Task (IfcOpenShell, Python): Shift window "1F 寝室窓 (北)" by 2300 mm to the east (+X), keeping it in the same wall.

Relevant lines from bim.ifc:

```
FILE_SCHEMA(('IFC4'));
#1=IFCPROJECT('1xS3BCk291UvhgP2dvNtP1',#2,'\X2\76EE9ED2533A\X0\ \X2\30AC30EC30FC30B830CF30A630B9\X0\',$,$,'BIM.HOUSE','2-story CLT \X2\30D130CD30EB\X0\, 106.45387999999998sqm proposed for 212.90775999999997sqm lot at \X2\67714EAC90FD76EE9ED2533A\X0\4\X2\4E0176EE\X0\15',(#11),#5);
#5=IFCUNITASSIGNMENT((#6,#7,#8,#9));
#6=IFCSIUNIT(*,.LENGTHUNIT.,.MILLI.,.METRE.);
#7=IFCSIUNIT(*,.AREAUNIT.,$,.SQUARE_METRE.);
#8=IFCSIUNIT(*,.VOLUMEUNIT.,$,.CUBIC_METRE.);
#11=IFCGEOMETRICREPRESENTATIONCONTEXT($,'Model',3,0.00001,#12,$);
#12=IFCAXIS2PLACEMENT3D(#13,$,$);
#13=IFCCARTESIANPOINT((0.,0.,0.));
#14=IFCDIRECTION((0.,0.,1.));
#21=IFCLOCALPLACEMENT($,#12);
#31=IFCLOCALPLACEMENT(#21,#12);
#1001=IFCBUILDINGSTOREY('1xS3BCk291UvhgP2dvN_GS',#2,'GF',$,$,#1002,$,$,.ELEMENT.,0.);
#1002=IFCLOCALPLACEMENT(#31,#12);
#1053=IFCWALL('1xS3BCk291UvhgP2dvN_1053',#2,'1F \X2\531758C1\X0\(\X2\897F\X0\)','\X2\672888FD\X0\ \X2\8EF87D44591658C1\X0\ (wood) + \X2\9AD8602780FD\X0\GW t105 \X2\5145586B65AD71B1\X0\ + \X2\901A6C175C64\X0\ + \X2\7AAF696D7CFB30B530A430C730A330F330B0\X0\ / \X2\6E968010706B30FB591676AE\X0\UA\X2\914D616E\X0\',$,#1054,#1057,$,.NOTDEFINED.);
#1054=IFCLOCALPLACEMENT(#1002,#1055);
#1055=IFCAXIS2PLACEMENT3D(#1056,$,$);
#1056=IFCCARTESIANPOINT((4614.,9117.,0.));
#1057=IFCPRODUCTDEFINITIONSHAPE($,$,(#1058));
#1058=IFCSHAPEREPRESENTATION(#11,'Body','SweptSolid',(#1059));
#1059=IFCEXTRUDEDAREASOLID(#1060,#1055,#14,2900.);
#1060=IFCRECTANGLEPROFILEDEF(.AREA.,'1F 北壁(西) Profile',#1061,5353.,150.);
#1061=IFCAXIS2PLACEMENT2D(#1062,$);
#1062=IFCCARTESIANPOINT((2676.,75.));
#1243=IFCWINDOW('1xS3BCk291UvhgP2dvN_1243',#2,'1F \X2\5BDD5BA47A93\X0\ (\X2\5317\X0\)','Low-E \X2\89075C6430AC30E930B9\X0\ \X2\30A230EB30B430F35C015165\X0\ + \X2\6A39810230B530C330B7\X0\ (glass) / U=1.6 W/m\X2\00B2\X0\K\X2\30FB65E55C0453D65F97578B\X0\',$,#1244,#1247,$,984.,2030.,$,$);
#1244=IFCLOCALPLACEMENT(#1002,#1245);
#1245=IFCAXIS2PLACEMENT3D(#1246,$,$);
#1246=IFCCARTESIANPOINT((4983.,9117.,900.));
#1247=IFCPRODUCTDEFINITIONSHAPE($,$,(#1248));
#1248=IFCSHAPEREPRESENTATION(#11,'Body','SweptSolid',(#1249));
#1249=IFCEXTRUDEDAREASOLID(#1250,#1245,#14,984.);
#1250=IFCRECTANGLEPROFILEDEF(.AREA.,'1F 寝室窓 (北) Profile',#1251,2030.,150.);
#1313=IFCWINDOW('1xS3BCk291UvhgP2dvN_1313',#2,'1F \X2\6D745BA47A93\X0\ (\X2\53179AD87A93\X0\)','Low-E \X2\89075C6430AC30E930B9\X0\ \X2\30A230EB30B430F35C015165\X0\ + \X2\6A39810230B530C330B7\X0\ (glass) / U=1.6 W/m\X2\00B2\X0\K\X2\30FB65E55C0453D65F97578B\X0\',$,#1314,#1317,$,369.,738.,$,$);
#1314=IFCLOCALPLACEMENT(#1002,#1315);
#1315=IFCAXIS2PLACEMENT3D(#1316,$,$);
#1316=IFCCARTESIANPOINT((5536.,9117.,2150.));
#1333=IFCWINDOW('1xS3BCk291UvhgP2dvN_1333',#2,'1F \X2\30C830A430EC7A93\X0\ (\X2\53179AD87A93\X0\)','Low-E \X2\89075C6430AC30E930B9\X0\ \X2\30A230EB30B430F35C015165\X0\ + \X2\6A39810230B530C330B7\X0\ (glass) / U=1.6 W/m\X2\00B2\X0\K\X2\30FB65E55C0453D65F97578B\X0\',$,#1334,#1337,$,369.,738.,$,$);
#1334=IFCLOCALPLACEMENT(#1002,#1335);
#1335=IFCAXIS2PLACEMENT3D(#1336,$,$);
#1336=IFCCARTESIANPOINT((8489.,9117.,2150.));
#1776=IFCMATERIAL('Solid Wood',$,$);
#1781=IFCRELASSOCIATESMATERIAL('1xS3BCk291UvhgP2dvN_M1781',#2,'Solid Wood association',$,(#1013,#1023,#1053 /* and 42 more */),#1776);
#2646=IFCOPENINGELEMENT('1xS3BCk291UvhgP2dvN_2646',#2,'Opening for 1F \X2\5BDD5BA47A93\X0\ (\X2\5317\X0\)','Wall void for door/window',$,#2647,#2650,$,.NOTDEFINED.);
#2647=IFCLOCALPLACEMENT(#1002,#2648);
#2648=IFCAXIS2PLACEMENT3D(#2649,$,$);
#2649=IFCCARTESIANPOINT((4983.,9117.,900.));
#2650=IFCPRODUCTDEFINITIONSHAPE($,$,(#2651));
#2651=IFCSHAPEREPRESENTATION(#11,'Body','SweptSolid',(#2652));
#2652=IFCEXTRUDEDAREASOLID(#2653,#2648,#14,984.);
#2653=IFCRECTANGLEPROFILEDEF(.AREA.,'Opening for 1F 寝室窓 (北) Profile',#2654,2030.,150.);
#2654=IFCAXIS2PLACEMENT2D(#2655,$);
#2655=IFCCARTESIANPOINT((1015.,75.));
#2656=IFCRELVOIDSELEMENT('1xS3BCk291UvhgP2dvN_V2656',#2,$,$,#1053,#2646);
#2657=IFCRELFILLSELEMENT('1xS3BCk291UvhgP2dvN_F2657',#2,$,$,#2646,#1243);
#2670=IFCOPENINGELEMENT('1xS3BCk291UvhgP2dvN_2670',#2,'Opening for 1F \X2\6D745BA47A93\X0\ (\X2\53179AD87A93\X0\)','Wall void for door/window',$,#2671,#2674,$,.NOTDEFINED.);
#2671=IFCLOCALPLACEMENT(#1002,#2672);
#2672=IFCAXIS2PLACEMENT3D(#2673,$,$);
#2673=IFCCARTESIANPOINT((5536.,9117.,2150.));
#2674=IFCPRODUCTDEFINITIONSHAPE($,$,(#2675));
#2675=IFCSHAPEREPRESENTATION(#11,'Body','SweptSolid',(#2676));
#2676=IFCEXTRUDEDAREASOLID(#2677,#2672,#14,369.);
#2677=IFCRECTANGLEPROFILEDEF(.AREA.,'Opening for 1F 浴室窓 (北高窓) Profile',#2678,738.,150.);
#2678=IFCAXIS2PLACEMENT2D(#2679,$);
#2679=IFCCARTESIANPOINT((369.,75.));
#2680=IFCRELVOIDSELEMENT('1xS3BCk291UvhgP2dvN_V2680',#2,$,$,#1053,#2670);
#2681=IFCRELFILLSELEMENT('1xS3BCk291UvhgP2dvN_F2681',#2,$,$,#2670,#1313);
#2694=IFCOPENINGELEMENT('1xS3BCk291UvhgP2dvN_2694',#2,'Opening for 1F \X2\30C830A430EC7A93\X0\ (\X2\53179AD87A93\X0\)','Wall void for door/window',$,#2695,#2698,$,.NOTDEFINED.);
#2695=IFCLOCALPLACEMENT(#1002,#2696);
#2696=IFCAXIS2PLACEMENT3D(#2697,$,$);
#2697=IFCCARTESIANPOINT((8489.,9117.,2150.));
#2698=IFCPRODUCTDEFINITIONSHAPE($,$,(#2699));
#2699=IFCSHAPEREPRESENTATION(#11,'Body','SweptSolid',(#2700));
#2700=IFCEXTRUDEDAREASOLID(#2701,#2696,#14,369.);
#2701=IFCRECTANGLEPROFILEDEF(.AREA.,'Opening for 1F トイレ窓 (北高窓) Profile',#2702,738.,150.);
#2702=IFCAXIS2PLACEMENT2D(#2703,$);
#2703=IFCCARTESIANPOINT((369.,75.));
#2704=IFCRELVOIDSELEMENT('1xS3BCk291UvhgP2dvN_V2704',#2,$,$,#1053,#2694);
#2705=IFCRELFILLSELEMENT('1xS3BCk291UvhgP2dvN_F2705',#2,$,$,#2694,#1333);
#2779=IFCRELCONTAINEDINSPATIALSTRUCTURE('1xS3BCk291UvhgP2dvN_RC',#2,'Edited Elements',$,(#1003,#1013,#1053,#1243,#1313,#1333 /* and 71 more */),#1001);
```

```python
import ifcopenshell
import ifcopenshell.api.geometry
import ifcopenshell.util.placement

model = ifcopenshell.open("bim.ifc")

window = model.by_guid("1xS3BCk291UvhgP2dvN_1243")
opening = window.FillsVoids[0].RelatingOpeningElement
wall = opening.VoidsElements[0].RelatingBuildingElement

wall_matrix = ifcopenshell.util.placement.get_local_placement(wall.ObjectPlacement)
shift = wall_matrix[:3, 0] * 2300.0
before = ifcopenshell.util.placement.get_local_placement(window.ObjectPlacement)[:3, 3].copy()

# The window is not placed relative to its opening, so move both.
for product in (opening, window):
    matrix = ifcopenshell.util.placement.get_local_placement(product.ObjectPlacement)
    matrix[:3, 3] += shift
    ifcopenshell.api.geometry.edit_object_placement(model, product=product, matrix=matrix, is_si=False)

after = ifcopenshell.util.placement.get_local_placement(window.ObjectPlacement)[:3, 3]
print("window moved by", (after - before).round(3) + 0.0)

model.write("bim_rev.ifc")
```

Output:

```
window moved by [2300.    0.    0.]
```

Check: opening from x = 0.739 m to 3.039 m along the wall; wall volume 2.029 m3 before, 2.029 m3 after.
